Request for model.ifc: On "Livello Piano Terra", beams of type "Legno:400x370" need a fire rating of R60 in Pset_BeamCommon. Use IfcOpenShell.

First a look at what the model holds.

```python
import ifcopenshell
import ifcopenshell.util.element

model = ifcopenshell.open("model.ifc")
print(model.schema)
storey = next(s for s in model.by_type("IfcBuildingStorey") if s.Name == "Livello Piano Terra")
beams = [e for e in ifcopenshell.util.element.get_decomposition(storey) if e.is_a("IfcBeam")]
seen = {}
for e in beams:
    element_type = ifcopenshell.util.element.get_type(e)
    key = (element_type.Name if element_type != e and element_type else None, ifcopenshell.util.element.get_pset(e, "Pset_BeamCommon", "FireRating"))
    seen[key] = seen.get(key, 0) + 1
for (name, value), count in sorted(seen.items(), key=str):
    print(count, "x", name, "|", value)
```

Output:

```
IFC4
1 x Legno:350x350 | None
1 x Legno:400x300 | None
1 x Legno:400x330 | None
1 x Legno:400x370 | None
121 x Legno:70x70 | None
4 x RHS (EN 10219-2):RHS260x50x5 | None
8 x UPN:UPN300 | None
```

```python
import ifcopenshell
import ifcopenshell.api.pset
import ifcopenshell.util.element

model = ifcopenshell.open("model.ifc")

storey = next(s for s in model.by_type("IfcBuildingStorey") if s.Name == "Livello Piano Terra")
beams = [e for e in ifcopenshell.util.element.get_decomposition(storey) if e.is_a("IfcBeam")]

count = 0
for e in beams:
    element_type = ifcopenshell.util.element.get_type(e)
    if element_type in (None, e) or element_type.Name != "Legno:400x370":
        continue
    # add_pset returns the element's existing set when there is one.
    pset = ifcopenshell.api.pset.add_pset(model, product=e, name="Pset_BeamCommon")
    ifcopenshell.api.pset.edit_pset(model, pset=pset, properties={"FireRating": "R60"})
    count += 1

print(count, "beams updated")

model.write("model_rev.ifc")
```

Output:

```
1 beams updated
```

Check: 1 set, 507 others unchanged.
